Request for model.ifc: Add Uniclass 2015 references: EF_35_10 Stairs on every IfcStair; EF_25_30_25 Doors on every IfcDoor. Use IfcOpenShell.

First a look at what the model holds.

```python
import ifcopenshell

model = ifcopenshell.open("model.ifc")
print(model.schema)
print("classifications:", [c.Name for c in model.by_type("IfcClassification")])
for ifc_class in ("IfcDoor", "IfcRoof", "IfcStair", "IfcWall", "IfcWindow"):
    print(ifc_class, len(model.by_type(ifc_class)))
```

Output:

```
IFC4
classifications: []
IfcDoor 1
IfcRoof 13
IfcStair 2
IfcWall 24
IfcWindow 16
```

```python
import ifcopenshell
import ifcopenshell.api.classification

model = ifcopenshell.open("model.ifc")

system = ifcopenshell.api.classification.add_classification(model, classification="Uniclass 2015")

codes = {
    "IfcStair": ("EF_35_10", "Stairs"),
    "IfcDoor": ("EF_25_30_25", "Doors"),
}
for ifc_class, (code, name) in codes.items():
    products = model.by_type(ifc_class)
    ifcopenshell.api.classification.add_reference(
        model, products=products, classification=system, identification=code, name=name
    )
    print(code, len(products))

model.write("model_rev.ifc")
```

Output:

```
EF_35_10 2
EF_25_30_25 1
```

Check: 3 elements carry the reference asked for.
